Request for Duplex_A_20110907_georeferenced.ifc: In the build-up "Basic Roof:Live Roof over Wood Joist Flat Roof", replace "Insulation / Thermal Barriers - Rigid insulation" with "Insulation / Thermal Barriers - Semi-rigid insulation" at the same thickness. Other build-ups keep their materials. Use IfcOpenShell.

First a look at what the model holds.

```python
import ifcopenshell
import ifcopenshell.util.element

model = ifcopenshell.open("Duplex_A_20110907_georeferenced.ifc")
print(model.schema)
for layer_set in model.by_type("IfcMaterialLayerSet"):
    if layer_set.LayerSetName == "Basic Roof:Live Roof over Wood Joist Flat Roof":
        for layer in layer_set.MaterialLayers:
            print(layer.id(), layer.Material and layer.Material.Name, layer.LayerThickness, sep=" | ")
        print(len(ifcopenshell.util.element.get_elements_by_material(model, layer_set)), "elements and types use it")
print(sorted(m.Name for m in model.by_type("IfcMaterial") if m.Name)[:60])
```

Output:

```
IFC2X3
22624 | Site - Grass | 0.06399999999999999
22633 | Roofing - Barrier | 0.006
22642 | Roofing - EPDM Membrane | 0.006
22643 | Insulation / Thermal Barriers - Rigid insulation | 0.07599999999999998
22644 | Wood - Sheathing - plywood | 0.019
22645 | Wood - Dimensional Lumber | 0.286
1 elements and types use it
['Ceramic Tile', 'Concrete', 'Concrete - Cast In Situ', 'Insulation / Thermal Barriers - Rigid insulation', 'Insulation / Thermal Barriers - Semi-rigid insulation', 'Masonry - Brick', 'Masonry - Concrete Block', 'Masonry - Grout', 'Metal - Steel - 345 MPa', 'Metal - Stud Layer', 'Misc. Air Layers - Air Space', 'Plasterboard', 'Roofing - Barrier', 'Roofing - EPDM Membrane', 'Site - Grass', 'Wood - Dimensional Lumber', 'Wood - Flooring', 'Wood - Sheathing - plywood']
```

```python
import ifcopenshell
import ifcopenshell.api.material

model = ifcopenshell.open("Duplex_A_20110907_georeferenced.ifc")

layer_set = next(s for s in model.by_type("IfcMaterialLayerSet") if s.LayerSetName == "Basic Roof:Live Roof over Wood Joist Flat Roof")
layer = next(l for l in layer_set.MaterialLayers if l.Material and l.Material.Name == "Insulation / Thermal Barriers - Rigid insulation")
material = next(m for m in model.by_type("IfcMaterial") if m.Name == "Insulation / Thermal Barriers - Semi-rigid insulation")

# Point this one layer at the other material; renaming the old one would change it everywhere.
ifcopenshell.api.material.edit_layer(model, layer=layer, attributes={}, material=material)

print([l.Material.Name if l.Material else None for l in layer_set.MaterialLayers])

model.write("Duplex_A_20110907_georeferenced_rev.ifc")
```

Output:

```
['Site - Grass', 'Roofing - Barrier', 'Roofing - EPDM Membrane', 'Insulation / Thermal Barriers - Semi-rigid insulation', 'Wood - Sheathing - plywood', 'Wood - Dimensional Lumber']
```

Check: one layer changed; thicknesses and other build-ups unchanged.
